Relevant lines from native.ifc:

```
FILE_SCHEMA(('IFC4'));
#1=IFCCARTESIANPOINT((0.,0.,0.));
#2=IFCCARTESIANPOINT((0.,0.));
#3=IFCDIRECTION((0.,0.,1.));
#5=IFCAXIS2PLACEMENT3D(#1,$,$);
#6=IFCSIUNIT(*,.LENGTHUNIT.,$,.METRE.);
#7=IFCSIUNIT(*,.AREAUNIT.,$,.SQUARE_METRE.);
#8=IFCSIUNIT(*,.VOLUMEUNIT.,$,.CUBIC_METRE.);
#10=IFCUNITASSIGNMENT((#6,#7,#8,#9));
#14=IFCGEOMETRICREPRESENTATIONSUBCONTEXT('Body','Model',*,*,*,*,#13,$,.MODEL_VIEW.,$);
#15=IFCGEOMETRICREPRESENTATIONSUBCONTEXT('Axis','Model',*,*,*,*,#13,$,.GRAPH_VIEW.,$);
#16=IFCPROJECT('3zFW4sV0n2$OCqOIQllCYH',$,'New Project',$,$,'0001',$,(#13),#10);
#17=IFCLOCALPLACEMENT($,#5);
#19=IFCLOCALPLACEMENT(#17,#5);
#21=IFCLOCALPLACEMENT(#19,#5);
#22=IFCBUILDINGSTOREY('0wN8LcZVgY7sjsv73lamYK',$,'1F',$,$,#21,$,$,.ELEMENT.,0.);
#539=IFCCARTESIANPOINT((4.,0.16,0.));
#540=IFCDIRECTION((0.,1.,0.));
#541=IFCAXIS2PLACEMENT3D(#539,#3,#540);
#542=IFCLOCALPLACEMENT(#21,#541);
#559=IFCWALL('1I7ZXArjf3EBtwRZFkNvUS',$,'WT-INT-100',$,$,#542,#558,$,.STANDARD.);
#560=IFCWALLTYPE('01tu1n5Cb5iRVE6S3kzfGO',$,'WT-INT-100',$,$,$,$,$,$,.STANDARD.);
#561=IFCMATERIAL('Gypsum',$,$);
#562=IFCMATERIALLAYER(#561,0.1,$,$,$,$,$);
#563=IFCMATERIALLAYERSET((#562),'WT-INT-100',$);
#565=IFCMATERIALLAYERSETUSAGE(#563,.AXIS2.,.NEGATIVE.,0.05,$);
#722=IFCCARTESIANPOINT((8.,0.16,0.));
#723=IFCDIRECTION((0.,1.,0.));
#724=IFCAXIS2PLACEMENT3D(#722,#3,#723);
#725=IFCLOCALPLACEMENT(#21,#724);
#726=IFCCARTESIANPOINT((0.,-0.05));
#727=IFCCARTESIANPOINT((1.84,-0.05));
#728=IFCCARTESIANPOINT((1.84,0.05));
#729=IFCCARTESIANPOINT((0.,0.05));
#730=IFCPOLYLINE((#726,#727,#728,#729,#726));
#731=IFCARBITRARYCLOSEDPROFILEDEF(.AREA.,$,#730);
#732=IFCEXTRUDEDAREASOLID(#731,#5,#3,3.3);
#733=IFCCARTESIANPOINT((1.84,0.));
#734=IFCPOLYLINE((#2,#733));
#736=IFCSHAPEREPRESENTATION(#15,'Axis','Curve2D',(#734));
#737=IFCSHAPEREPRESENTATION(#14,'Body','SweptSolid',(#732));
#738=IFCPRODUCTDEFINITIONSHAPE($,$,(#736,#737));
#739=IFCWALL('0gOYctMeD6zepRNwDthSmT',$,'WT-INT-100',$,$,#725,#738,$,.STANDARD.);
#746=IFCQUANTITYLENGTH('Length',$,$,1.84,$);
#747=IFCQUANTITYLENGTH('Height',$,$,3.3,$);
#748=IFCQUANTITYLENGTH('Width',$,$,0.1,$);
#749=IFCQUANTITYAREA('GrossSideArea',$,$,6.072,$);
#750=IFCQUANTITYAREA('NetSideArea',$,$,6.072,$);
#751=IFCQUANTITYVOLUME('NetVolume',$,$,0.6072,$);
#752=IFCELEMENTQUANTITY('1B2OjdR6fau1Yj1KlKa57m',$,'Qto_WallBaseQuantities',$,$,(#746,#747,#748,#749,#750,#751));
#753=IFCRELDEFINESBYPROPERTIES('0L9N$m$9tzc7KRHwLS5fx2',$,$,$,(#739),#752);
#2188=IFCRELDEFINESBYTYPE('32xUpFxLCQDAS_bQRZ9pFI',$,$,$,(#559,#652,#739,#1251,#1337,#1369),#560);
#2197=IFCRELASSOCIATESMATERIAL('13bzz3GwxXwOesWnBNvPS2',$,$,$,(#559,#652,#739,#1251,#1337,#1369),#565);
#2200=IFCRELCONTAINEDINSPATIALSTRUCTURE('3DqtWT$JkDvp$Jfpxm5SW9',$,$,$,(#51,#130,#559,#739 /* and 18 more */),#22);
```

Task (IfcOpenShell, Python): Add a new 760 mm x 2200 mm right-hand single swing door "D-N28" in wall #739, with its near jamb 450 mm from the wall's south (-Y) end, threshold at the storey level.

```python
import numpy as np
import ifcopenshell
import ifcopenshell.api.feature
import ifcopenshell.api.geometry
import ifcopenshell.api.pset
import ifcopenshell.api.root
import ifcopenshell.api.spatial
import ifcopenshell.geom
import ifcopenshell.util.element
import ifcopenshell.util.placement
import ifcopenshell.util.representation
import ifcopenshell.util.shape
import ifcopenshell.util.unit

model = ifcopenshell.open("native.ifc")
unit_scale = ifcopenshell.util.unit.calculate_unit_scale(model)
area_scale = ifcopenshell.util.unit.calculate_unit_scale(model, "AREAUNIT")
volume_scale = ifcopenshell.util.unit.calculate_unit_scale(model, "VOLUMEUNIT")
settings = ifcopenshell.geom.settings()


def volume(element):
    """Net volume in cubic metres, openings subtracted."""
    shape = ifcopenshell.geom.create_shape(settings, element)
    return ifcopenshell.util.shape.get_volume(shape.geometry)


wall = model.by_id(739)
storey = ifcopenshell.util.element.get_container(wall, ifc_class="IfcBuildingStorey")
context = ifcopenshell.util.representation.get_context(model, "Model", "Body", "MODEL_VIEW")
before = volume(wall)

width, height, from_end, sill = 0.76, 2.2, 0.45, 0.0  # metres

# The wall runs along its own X axis, and the end named is its -X end.
wall_shape = ifcopenshell.geom.create_shape(settings, wall)
x, y, z = ifcopenshell.util.shape.get_vertices(wall_shape.geometry).T
start = x.min() + from_end
face, thickness = float(y.min()), float(y.max() - y.min())
wall_matrix = ifcopenshell.util.placement.get_local_placement(wall.ObjectPlacement)
level = ifcopenshell.util.placement.get_local_placement(storey.ObjectPlacement)[2, 3]


def in_wall(x, y):
    """Placement at x, y metres in the wall's axes, at sill height."""
    matrix = wall_matrix.copy()
    matrix[:, 3] = wall_matrix @ np.array([x / unit_scale, y / unit_scale, 0.0, 1.0])
    matrix[2, 3] = level + sill / unit_scale
    return matrix


# Opening: a box that overshoots both wall faces by 50 mm.
opening = ifcopenshell.api.root.create_entity(model, ifc_class="IfcOpeningElement", predefined_type="OPENING")
box = ifcopenshell.api.geometry.add_wall_representation(
    model, context=context, length=width, height=height, thickness=thickness + 0.1
)
ifcopenshell.api.geometry.assign_representation(model, product=opening, representation=box)
ifcopenshell.api.geometry.edit_object_placement(model, product=opening, matrix=in_wall(start, face - 0.05), is_si=False)
ifcopenshell.api.feature.add_feature(model, feature=opening, element=wall)

door = ifcopenshell.api.root.create_entity(model, ifc_class="IfcDoor", name="D-N28", predefined_type="DOOR")
door.OverallWidth, door.OverallHeight = width / unit_scale, height / unit_scale
door.OperationType = "SINGLE_SWING_RIGHT"
body = ifcopenshell.api.geometry.add_door_representation(
    model,
    context=context,
    overall_width=door.OverallWidth,
    overall_height=door.OverallHeight,
    operation_type="SINGLE_SWING_RIGHT",
    lining_properties={"LiningDepth": thickness / unit_scale, "ThresholdDepth": thickness / unit_scale},
)
ifcopenshell.api.geometry.assign_representation(model, product=door, representation=body)
ifcopenshell.api.spatial.assign_container(model, products=[door], relating_structure=storey)
ifcopenshell.api.feature.add_filling(model, opening=opening, element=door)

# The lining spans the wall, so the door starts at the wall face.
ifcopenshell.api.geometry.edit_object_placement(model, product=door, matrix=in_wall(start, face), is_si=False)

after = volume(wall)

# Update the wall's stored quantities.
qto = model.by_id(ifcopenshell.util.element.get_pset(wall, "Qto_WallBaseQuantities", should_inherit=False)["id"])
ifcopenshell.api.pset.edit_qto(model, qto=qto, properties={
    "NetSideArea": after / thickness / area_scale,
    "NetVolume": after / volume_scale,
})

print(f"wall volume {before:.3f} -> {after:.3f} m3")

model.write("native-out.ifc")
```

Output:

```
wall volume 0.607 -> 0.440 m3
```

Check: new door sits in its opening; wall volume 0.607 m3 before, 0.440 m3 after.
